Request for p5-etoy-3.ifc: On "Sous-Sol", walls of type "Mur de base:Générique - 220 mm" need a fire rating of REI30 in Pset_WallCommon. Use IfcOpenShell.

First a look at what the model holds.

```python
import ifcopenshell
import ifcopenshell.util.element

model = ifcopenshell.open("p5-etoy-3.ifc")
print(model.schema)
storey = next(s for s in model.by_type("IfcBuildingStorey") if s.Name == "Sous-Sol")
walls = [e for e in ifcopenshell.util.element.get_decomposition(storey) if e.is_a("IfcWall")]
seen = {}
for e in walls:
    element_type = ifcopenshell.util.element.get_type(e)
    key = (element_type.Name if element_type != e and element_type else None, ifcopenshell.util.element.get_pset(e, "Pset_WallCommon", "FireRating"))
    seen[key] = seen.get(key, 0) + 1
for (name, value), count in sorted(seen.items(), key=str):
    print(count, "x", name, "|", value)
```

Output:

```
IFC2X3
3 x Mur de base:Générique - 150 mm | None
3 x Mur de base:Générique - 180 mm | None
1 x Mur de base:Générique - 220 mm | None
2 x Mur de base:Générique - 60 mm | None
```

```python
import ifcopenshell
import ifcopenshell.api.pset
import ifcopenshell.util.element

model = ifcopenshell.open("p5-etoy-3.ifc")

storey = next(s for s in model.by_type("IfcBuildingStorey") if s.Name == "Sous-Sol")
walls = [e for e in ifcopenshell.util.element.get_decomposition(storey) if e.is_a("IfcWall")]

count = 0
for e in walls:
    element_type = ifcopenshell.util.element.get_type(e)
    if element_type in (None, e) or element_type.Name != "Mur de base:Générique - 220 mm":
        continue
    # add_pset returns the element's existing set when there is one.
    pset = ifcopenshell.api.pset.add_pset(model, product=e, name="Pset_WallCommon")
    ifcopenshell.api.pset.edit_pset(model, pset=pset, properties={"FireRating": "REI30"})
    count += 1

print(count, "walls updated")

model.write("p5-etoy-3_rev.ifc")
```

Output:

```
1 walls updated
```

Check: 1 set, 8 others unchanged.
